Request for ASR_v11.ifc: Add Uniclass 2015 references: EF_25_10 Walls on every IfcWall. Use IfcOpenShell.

First a look at what the model holds.

```python
import ifcopenshell

model = ifcopenshell.open("ASR_v11.ifc")
print(model.schema)
print("classifications:", [c.Name for c in model.by_type("IfcClassification")])
for ifc_class in ("IfcDoor", "IfcRoof", "IfcStair", "IfcWall", "IfcWindow"):
    print(ifc_class, len(model.by_type(ifc_class)))
```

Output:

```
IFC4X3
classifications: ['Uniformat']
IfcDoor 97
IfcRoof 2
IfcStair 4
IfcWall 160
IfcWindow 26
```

```python
import ifcopenshell
import ifcopenshell.api.classification

model = ifcopenshell.open("ASR_v11.ifc")

system = ifcopenshell.api.classification.add_classification(model, classification="Uniclass 2015")

codes = {
    "IfcWall": ("EF_25_10", "Walls"),
}
for ifc_class, (code, name) in codes.items():
    products = model.by_type(ifc_class)
    ifcopenshell.api.classification.add_reference(
        model, products=products, classification=system, identification=code, name=name
    )
    print(code, len(products))

model.write("ASR_v11_updated.ifc")
```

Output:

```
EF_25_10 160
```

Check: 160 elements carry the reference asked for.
